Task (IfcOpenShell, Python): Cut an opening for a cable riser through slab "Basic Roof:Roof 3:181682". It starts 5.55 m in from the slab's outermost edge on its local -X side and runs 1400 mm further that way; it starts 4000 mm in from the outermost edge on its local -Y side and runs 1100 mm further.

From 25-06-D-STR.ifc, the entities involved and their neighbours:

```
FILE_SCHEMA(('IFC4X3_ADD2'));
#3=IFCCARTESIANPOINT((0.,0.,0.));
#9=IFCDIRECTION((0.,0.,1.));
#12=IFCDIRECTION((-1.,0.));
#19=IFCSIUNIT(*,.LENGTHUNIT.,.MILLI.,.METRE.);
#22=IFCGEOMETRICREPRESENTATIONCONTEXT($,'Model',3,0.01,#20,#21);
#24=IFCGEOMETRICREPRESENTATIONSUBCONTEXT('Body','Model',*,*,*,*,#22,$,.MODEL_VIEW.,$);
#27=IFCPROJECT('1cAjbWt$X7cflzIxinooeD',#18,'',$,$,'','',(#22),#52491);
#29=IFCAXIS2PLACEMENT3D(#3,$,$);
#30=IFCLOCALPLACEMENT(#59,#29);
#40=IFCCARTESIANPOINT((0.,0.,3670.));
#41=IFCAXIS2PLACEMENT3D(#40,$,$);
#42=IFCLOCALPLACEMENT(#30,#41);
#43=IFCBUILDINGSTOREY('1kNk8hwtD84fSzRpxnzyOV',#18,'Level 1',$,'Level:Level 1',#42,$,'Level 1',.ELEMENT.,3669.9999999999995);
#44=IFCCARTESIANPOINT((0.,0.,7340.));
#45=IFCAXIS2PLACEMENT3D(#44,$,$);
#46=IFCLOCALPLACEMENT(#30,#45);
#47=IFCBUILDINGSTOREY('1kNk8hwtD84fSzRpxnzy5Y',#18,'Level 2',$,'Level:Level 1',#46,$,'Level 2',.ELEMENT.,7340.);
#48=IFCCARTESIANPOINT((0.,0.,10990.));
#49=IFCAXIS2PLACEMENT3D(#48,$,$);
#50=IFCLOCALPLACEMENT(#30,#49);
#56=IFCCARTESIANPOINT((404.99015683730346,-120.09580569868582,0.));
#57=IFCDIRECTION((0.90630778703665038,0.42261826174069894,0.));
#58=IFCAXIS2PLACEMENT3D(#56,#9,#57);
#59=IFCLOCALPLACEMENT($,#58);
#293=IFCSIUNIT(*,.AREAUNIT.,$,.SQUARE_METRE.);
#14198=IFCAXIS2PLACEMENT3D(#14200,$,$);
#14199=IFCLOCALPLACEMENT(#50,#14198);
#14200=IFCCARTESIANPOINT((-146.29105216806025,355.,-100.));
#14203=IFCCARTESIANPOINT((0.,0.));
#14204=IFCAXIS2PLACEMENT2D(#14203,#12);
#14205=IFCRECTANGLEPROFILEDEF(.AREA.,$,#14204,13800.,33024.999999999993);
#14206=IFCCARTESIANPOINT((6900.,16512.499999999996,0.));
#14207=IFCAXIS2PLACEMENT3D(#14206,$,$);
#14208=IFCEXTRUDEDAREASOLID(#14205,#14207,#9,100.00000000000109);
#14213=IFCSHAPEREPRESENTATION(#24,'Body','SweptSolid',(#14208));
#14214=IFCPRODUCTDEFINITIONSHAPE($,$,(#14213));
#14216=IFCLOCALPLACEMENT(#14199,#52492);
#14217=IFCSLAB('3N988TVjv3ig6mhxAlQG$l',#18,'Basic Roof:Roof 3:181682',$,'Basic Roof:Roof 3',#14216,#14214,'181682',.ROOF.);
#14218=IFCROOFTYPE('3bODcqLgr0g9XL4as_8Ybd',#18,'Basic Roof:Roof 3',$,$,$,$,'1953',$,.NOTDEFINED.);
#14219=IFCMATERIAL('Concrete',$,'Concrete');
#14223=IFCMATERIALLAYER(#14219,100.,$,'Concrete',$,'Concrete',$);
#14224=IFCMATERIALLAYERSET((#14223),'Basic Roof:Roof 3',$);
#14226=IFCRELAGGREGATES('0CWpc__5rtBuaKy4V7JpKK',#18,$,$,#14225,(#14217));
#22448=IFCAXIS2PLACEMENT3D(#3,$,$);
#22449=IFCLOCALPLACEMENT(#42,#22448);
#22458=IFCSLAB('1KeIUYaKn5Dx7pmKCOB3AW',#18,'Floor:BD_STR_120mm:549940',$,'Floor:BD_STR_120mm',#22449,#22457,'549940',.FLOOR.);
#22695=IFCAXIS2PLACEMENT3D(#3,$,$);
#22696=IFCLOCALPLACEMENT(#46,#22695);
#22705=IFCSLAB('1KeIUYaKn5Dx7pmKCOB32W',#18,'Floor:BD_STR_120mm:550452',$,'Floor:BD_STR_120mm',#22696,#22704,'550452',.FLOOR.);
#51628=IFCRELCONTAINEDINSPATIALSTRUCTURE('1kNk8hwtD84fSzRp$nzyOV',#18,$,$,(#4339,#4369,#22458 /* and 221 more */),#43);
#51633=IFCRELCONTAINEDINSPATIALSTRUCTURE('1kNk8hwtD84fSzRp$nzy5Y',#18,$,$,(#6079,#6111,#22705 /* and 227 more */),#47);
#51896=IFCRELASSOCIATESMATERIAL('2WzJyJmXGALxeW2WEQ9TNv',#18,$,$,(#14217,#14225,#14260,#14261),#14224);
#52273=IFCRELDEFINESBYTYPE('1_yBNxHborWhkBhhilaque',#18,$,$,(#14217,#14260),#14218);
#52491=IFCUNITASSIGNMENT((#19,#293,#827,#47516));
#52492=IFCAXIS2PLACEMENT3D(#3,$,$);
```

```python
import numpy as np
import ifcopenshell
import ifcopenshell.api.feature
import ifcopenshell.api.geometry
import ifcopenshell.api.root
import ifcopenshell.geom
import ifcopenshell.util.placement
import ifcopenshell.util.representation
import ifcopenshell.util.shape
import ifcopenshell.util.unit

model = ifcopenshell.open("25-06-D-STR.ifc")
unit_scale = ifcopenshell.util.unit.calculate_unit_scale(model)
settings = ifcopenshell.geom.settings()


def volume(element):
    """Net volume in cubic metres, openings subtracted."""
    shape = ifcopenshell.geom.create_shape(settings, element)
    return ifcopenshell.util.shape.get_volume(shape.geometry)


slab = model.by_guid("3N988TVjv3ig6mhxAlQG$l")
before = volume(slab)

# Extent in the slab's own axes, in metres. The edges named are its -X and -Y sides.
slab_shape = ifcopenshell.geom.create_shape(settings, slab)
vertices = ifcopenshell.util.shape.get_vertices(slab_shape.geometry)
x_min, y_min, bottom = vertices.min(axis=0)
top = vertices[:, 2].max()

opening = ifcopenshell.api.root.create_entity(model, ifc_class="IfcOpeningElement", name="Cable riser opening", predefined_type="OPENING")
context = ifcopenshell.util.representation.get_context(model, "Model", "Body", "MODEL_VIEW")
width, depth = 1.4, 1.1
outline = [(0.0, 0.0), (width, 0.0), (width, depth), (0.0, depth), (0.0, 0.0)]
# Overshoot both faces by 50 mm so the cut is clean.
shape = ifcopenshell.api.geometry.add_slab_representation(
    model, context=context, depth=top - bottom + 0.1, polyline=outline
)
ifcopenshell.api.geometry.assign_representation(model, product=opening, representation=shape)

matrix = ifcopenshell.util.placement.get_local_placement(slab.ObjectPlacement)
matrix[:, 3] = matrix @ np.append(np.array([x_min + 5.55, y_min + 4, bottom - 0.05]) / unit_scale, 1.0)
ifcopenshell.api.geometry.edit_object_placement(model, product=opening, matrix=matrix, is_si=False)
ifcopenshell.api.feature.add_feature(model, feature=opening, element=slab)

after = volume(slab)

print(f"slab volume {before:.3f} -> {after:.3f} m3")

model.write("25-06-D-STR_v2.ifc")
```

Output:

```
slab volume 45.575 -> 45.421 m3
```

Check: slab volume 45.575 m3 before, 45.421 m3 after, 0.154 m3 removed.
